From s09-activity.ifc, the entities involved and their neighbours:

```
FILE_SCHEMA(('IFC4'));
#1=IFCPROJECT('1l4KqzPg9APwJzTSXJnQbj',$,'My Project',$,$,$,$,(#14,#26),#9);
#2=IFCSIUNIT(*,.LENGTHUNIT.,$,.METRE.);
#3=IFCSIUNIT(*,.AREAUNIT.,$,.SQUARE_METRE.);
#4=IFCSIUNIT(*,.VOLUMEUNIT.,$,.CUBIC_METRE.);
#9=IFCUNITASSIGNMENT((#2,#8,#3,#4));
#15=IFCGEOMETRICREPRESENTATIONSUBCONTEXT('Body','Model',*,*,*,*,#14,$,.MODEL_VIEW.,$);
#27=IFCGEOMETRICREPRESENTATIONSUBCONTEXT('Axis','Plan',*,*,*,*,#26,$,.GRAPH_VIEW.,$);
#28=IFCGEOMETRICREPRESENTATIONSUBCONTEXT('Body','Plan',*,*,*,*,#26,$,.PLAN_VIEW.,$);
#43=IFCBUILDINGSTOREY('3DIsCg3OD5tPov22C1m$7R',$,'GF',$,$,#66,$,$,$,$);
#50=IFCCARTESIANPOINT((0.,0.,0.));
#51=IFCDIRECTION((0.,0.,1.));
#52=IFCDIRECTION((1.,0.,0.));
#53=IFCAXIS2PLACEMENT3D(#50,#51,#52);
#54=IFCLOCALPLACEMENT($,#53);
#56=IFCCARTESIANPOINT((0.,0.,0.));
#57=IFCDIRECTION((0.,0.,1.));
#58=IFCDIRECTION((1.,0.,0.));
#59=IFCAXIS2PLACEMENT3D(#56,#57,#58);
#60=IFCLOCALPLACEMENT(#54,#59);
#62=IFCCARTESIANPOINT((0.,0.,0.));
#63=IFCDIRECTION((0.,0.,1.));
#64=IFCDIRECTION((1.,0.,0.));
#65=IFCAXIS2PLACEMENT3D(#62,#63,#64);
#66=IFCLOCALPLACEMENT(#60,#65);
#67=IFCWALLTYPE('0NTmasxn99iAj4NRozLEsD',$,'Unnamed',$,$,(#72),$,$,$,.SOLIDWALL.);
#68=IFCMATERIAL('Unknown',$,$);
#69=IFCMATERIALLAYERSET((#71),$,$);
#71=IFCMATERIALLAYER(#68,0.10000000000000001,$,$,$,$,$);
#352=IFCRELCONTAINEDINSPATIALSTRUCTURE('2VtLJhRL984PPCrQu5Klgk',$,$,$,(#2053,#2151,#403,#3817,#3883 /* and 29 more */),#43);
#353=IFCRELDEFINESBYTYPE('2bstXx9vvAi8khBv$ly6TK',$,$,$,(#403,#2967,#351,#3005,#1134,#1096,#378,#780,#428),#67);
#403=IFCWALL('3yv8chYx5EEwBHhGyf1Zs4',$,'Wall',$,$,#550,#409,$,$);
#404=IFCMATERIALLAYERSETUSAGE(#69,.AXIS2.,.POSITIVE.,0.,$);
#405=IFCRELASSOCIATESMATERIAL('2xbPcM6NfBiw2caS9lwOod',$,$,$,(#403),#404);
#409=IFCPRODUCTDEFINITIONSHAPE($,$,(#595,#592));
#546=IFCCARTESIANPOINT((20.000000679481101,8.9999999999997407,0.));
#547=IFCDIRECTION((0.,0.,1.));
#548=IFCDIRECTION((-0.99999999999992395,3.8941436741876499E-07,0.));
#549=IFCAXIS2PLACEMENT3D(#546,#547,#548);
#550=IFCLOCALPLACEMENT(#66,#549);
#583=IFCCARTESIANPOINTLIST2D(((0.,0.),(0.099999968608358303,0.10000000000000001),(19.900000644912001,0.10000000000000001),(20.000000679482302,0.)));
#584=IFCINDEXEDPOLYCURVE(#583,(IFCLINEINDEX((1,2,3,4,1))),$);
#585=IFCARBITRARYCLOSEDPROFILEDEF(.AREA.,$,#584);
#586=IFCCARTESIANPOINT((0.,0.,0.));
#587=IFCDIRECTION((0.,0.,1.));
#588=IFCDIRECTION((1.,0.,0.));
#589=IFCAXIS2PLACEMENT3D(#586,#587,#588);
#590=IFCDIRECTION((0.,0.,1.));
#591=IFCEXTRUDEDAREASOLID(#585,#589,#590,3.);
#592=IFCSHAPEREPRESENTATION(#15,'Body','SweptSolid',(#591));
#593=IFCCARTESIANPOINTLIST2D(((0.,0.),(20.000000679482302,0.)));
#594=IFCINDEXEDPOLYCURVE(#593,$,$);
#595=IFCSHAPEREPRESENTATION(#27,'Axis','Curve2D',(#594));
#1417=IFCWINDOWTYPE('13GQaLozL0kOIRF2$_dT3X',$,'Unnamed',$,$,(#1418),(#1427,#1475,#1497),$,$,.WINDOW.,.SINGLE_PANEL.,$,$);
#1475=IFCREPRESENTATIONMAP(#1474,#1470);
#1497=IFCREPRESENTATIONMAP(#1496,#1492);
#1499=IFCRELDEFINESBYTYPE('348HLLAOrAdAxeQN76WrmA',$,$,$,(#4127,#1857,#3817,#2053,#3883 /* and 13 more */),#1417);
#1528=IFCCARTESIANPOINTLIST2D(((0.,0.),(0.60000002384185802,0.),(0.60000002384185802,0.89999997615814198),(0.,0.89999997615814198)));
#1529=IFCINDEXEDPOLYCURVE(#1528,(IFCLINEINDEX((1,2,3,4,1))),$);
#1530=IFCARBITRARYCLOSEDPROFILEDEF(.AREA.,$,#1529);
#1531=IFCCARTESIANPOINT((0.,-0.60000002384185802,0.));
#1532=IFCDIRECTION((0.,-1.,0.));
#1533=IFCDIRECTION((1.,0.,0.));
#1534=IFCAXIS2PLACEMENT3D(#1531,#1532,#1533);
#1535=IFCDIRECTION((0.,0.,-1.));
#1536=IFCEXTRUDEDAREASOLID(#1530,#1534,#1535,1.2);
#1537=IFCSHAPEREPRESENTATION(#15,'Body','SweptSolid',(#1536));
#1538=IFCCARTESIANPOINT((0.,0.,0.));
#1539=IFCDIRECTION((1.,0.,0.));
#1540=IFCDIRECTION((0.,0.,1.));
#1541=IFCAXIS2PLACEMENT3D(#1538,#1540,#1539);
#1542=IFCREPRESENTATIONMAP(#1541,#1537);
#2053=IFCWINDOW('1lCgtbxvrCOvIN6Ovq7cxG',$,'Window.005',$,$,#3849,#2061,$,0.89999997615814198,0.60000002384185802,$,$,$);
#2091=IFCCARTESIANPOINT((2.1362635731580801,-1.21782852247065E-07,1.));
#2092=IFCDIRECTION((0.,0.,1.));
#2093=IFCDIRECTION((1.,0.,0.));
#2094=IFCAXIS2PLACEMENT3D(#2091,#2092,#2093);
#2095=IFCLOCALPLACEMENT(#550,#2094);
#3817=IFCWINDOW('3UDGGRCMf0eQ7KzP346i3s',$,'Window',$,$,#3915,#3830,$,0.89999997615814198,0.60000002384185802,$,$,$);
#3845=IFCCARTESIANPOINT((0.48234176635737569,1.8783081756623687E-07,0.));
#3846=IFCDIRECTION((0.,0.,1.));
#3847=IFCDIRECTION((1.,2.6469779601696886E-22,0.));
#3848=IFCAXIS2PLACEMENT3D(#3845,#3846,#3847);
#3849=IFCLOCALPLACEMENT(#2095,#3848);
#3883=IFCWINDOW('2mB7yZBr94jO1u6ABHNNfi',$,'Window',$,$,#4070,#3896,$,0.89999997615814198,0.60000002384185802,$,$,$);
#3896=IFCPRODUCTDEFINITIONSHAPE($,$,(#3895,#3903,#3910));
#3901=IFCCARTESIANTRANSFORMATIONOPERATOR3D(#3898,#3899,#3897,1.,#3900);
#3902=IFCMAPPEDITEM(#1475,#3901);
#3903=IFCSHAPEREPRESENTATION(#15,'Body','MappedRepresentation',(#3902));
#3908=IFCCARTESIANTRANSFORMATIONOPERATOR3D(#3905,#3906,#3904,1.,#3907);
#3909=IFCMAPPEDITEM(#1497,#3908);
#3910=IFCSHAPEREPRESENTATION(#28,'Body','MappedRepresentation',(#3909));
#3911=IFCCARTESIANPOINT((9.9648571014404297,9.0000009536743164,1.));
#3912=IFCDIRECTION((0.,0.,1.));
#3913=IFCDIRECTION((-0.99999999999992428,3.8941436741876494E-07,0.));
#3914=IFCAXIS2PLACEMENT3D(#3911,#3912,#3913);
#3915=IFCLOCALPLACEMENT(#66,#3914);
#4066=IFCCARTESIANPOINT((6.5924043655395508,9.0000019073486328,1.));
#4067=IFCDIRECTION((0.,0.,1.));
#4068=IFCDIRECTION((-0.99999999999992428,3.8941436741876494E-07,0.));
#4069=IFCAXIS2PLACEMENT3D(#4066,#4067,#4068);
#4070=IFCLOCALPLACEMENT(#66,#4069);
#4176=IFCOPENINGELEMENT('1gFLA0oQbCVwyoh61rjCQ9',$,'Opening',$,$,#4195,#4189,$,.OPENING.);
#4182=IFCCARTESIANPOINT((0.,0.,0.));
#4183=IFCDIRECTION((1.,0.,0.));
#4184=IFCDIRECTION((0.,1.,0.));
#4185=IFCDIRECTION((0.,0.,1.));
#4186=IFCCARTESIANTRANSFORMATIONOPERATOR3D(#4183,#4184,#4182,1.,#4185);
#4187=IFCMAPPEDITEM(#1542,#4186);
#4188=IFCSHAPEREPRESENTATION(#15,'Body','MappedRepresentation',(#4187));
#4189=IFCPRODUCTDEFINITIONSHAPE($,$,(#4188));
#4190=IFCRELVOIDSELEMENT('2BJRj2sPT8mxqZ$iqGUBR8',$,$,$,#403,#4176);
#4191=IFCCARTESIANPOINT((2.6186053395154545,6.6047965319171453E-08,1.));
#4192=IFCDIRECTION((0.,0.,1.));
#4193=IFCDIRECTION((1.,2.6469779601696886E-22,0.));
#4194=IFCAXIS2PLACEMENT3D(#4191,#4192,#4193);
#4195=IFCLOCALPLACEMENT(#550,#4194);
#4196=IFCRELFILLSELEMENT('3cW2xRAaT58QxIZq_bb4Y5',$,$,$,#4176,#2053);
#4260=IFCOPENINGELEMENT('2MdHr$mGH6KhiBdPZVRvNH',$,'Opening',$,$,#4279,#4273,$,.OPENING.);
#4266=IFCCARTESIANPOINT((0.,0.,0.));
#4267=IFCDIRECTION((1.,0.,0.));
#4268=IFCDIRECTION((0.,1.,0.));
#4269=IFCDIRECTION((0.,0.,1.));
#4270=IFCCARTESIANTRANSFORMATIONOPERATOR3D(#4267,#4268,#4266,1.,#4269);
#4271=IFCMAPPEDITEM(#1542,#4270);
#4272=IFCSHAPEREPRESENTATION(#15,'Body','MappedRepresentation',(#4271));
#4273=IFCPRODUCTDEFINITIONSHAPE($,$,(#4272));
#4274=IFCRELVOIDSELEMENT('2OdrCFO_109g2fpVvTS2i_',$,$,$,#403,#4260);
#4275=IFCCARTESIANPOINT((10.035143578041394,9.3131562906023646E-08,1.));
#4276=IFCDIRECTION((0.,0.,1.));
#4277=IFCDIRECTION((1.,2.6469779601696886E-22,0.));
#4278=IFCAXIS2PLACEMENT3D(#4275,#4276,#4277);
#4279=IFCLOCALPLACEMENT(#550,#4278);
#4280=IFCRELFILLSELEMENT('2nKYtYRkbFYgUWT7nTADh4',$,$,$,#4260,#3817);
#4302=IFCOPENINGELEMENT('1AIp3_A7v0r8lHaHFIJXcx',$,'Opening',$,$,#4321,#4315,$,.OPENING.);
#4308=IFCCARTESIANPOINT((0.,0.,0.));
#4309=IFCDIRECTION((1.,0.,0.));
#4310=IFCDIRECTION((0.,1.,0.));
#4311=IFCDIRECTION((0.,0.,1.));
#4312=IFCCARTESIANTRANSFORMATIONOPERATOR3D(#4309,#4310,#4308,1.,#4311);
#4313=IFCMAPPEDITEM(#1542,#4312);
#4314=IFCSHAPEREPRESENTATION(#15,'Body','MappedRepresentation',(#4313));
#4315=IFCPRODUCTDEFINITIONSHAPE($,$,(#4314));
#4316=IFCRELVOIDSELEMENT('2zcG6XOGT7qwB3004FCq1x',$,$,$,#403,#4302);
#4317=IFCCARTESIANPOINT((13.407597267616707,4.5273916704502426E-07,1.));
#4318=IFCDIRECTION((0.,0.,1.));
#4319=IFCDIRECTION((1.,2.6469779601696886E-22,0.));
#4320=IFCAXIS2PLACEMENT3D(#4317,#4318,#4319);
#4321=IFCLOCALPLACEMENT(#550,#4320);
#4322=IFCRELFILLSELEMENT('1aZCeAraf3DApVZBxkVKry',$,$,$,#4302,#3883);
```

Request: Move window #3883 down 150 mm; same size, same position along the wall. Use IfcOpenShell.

```python
import numpy as np
import ifcopenshell
import ifcopenshell.api.geometry
import ifcopenshell.util.placement
import ifcopenshell.util.unit

model = ifcopenshell.open("s09-activity.ifc")
unit_scale = ifcopenshell.util.unit.calculate_unit_scale(model)

window = model.by_guid("2mB7yZBr94jO1u6ABHNNfi")
opening = window.FillsVoids[0].RelatingOpeningElement
dz = -0.15

shift = np.array([0.0, 0.0, dz])
# The window is not placed relative to its opening, so move both.
for product in (opening, window):
    matrix = ifcopenshell.util.placement.get_local_placement(product.ObjectPlacement)
    matrix[:3, 3] += shift
    ifcopenshell.api.geometry.edit_object_placement(model, product=product, matrix=matrix, is_si=False)

print(f"moved by {dz * unit_scale:+.3f} m")

model.write("s09-activity-out.ifc")
```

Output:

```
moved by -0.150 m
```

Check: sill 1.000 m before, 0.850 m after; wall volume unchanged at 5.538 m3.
